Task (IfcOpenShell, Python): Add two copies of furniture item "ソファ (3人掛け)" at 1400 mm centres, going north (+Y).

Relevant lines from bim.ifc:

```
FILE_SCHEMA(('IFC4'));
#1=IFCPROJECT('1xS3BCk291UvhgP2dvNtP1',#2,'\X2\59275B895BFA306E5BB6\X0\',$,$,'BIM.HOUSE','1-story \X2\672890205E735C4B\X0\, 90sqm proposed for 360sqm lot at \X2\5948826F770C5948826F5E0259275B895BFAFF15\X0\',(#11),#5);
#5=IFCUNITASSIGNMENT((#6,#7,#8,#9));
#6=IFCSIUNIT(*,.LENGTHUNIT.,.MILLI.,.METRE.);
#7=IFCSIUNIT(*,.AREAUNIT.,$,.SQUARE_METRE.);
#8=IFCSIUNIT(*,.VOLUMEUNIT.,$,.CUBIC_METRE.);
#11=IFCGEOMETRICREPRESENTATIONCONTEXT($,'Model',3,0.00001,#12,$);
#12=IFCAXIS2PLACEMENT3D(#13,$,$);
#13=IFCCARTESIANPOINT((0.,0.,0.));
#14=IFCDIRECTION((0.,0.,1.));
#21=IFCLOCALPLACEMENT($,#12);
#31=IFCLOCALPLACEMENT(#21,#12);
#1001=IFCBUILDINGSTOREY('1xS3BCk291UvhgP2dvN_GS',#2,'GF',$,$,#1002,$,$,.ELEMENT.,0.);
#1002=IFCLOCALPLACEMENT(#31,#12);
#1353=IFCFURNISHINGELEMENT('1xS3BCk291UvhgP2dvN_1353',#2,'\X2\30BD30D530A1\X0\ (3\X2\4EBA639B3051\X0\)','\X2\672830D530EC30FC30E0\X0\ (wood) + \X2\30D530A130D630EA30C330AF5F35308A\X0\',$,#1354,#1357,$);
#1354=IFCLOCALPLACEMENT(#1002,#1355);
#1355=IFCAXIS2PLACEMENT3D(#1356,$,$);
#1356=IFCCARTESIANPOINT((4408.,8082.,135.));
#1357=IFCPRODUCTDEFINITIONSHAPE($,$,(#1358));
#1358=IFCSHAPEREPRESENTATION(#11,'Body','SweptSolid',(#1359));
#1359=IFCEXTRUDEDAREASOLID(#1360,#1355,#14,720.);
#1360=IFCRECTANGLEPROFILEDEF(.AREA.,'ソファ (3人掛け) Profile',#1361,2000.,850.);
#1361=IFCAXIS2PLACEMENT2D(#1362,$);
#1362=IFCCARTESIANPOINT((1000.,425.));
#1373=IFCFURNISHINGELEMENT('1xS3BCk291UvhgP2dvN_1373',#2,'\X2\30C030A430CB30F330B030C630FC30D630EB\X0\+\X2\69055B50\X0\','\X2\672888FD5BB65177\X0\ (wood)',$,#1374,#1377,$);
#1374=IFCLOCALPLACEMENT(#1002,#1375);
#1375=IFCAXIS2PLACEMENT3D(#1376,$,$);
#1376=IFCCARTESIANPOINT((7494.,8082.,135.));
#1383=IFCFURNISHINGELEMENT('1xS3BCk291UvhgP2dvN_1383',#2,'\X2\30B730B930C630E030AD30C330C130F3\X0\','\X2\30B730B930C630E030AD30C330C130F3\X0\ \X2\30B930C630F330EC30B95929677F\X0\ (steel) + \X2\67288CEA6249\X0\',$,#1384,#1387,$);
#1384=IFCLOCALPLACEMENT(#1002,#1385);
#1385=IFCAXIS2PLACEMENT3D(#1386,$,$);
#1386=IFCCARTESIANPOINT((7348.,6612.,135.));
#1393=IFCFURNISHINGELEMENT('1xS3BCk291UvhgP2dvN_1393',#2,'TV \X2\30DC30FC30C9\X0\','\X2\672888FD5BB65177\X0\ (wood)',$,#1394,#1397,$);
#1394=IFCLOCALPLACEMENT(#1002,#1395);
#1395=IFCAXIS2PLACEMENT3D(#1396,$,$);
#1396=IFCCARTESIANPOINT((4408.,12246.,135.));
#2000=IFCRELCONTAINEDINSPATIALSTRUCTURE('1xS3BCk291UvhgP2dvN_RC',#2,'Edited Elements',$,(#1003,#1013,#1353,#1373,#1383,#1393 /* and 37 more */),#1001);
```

```python
import numpy as np
import ifcopenshell
import ifcopenshell.api.geometry
import ifcopenshell.api.root
import ifcopenshell.util.element
import ifcopenshell.util.placement
import ifcopenshell.util.unit

model = ifcopenshell.open("bim.ifc")
unit_scale = ifcopenshell.util.unit.calculate_unit_scale(model)


def reuse_history(source, copy):
    """copy_class also copies each property set's owner history, people and application; keep the originals."""
    for rel in copy.IsDefinedBy:
        if rel.is_a("IfcRelDefinesByProperties") and (history := rel.RelatingPropertyDefinition.OwnerHistory):
            rel.RelatingPropertyDefinition.OwnerHistory = source.OwnerHistory
            ifcopenshell.util.element.remove_deep2(model, history)


source = model.by_guid("1xS3BCk291UvhgP2dvN_1353")
base = ifcopenshell.util.placement.get_local_placement(source.ObjectPlacement)
step = np.array([0.0, 1.0, 0.0]) * 1.4 / unit_scale

for i in range(1, 3):
    copy = ifcopenshell.api.root.copy_class(model, product=source)
    copy.Representation = ifcopenshell.util.element.copy_deep(
        model, source.Representation, exclude=["IfcGeometricRepresentationContext", "IfcRepresentationMap"]
    )
    reuse_history(source, copy)
    matrix = base.copy()
    matrix[:3, 3] += i * step
    print("added at", matrix[:3, 3].round(3) + 0.0)
    ifcopenshell.api.geometry.edit_object_placement(model, product=copy, matrix=matrix, is_si=False)

model.write("bim-out.ifc")
```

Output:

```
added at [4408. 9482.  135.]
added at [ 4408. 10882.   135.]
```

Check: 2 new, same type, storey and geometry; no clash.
